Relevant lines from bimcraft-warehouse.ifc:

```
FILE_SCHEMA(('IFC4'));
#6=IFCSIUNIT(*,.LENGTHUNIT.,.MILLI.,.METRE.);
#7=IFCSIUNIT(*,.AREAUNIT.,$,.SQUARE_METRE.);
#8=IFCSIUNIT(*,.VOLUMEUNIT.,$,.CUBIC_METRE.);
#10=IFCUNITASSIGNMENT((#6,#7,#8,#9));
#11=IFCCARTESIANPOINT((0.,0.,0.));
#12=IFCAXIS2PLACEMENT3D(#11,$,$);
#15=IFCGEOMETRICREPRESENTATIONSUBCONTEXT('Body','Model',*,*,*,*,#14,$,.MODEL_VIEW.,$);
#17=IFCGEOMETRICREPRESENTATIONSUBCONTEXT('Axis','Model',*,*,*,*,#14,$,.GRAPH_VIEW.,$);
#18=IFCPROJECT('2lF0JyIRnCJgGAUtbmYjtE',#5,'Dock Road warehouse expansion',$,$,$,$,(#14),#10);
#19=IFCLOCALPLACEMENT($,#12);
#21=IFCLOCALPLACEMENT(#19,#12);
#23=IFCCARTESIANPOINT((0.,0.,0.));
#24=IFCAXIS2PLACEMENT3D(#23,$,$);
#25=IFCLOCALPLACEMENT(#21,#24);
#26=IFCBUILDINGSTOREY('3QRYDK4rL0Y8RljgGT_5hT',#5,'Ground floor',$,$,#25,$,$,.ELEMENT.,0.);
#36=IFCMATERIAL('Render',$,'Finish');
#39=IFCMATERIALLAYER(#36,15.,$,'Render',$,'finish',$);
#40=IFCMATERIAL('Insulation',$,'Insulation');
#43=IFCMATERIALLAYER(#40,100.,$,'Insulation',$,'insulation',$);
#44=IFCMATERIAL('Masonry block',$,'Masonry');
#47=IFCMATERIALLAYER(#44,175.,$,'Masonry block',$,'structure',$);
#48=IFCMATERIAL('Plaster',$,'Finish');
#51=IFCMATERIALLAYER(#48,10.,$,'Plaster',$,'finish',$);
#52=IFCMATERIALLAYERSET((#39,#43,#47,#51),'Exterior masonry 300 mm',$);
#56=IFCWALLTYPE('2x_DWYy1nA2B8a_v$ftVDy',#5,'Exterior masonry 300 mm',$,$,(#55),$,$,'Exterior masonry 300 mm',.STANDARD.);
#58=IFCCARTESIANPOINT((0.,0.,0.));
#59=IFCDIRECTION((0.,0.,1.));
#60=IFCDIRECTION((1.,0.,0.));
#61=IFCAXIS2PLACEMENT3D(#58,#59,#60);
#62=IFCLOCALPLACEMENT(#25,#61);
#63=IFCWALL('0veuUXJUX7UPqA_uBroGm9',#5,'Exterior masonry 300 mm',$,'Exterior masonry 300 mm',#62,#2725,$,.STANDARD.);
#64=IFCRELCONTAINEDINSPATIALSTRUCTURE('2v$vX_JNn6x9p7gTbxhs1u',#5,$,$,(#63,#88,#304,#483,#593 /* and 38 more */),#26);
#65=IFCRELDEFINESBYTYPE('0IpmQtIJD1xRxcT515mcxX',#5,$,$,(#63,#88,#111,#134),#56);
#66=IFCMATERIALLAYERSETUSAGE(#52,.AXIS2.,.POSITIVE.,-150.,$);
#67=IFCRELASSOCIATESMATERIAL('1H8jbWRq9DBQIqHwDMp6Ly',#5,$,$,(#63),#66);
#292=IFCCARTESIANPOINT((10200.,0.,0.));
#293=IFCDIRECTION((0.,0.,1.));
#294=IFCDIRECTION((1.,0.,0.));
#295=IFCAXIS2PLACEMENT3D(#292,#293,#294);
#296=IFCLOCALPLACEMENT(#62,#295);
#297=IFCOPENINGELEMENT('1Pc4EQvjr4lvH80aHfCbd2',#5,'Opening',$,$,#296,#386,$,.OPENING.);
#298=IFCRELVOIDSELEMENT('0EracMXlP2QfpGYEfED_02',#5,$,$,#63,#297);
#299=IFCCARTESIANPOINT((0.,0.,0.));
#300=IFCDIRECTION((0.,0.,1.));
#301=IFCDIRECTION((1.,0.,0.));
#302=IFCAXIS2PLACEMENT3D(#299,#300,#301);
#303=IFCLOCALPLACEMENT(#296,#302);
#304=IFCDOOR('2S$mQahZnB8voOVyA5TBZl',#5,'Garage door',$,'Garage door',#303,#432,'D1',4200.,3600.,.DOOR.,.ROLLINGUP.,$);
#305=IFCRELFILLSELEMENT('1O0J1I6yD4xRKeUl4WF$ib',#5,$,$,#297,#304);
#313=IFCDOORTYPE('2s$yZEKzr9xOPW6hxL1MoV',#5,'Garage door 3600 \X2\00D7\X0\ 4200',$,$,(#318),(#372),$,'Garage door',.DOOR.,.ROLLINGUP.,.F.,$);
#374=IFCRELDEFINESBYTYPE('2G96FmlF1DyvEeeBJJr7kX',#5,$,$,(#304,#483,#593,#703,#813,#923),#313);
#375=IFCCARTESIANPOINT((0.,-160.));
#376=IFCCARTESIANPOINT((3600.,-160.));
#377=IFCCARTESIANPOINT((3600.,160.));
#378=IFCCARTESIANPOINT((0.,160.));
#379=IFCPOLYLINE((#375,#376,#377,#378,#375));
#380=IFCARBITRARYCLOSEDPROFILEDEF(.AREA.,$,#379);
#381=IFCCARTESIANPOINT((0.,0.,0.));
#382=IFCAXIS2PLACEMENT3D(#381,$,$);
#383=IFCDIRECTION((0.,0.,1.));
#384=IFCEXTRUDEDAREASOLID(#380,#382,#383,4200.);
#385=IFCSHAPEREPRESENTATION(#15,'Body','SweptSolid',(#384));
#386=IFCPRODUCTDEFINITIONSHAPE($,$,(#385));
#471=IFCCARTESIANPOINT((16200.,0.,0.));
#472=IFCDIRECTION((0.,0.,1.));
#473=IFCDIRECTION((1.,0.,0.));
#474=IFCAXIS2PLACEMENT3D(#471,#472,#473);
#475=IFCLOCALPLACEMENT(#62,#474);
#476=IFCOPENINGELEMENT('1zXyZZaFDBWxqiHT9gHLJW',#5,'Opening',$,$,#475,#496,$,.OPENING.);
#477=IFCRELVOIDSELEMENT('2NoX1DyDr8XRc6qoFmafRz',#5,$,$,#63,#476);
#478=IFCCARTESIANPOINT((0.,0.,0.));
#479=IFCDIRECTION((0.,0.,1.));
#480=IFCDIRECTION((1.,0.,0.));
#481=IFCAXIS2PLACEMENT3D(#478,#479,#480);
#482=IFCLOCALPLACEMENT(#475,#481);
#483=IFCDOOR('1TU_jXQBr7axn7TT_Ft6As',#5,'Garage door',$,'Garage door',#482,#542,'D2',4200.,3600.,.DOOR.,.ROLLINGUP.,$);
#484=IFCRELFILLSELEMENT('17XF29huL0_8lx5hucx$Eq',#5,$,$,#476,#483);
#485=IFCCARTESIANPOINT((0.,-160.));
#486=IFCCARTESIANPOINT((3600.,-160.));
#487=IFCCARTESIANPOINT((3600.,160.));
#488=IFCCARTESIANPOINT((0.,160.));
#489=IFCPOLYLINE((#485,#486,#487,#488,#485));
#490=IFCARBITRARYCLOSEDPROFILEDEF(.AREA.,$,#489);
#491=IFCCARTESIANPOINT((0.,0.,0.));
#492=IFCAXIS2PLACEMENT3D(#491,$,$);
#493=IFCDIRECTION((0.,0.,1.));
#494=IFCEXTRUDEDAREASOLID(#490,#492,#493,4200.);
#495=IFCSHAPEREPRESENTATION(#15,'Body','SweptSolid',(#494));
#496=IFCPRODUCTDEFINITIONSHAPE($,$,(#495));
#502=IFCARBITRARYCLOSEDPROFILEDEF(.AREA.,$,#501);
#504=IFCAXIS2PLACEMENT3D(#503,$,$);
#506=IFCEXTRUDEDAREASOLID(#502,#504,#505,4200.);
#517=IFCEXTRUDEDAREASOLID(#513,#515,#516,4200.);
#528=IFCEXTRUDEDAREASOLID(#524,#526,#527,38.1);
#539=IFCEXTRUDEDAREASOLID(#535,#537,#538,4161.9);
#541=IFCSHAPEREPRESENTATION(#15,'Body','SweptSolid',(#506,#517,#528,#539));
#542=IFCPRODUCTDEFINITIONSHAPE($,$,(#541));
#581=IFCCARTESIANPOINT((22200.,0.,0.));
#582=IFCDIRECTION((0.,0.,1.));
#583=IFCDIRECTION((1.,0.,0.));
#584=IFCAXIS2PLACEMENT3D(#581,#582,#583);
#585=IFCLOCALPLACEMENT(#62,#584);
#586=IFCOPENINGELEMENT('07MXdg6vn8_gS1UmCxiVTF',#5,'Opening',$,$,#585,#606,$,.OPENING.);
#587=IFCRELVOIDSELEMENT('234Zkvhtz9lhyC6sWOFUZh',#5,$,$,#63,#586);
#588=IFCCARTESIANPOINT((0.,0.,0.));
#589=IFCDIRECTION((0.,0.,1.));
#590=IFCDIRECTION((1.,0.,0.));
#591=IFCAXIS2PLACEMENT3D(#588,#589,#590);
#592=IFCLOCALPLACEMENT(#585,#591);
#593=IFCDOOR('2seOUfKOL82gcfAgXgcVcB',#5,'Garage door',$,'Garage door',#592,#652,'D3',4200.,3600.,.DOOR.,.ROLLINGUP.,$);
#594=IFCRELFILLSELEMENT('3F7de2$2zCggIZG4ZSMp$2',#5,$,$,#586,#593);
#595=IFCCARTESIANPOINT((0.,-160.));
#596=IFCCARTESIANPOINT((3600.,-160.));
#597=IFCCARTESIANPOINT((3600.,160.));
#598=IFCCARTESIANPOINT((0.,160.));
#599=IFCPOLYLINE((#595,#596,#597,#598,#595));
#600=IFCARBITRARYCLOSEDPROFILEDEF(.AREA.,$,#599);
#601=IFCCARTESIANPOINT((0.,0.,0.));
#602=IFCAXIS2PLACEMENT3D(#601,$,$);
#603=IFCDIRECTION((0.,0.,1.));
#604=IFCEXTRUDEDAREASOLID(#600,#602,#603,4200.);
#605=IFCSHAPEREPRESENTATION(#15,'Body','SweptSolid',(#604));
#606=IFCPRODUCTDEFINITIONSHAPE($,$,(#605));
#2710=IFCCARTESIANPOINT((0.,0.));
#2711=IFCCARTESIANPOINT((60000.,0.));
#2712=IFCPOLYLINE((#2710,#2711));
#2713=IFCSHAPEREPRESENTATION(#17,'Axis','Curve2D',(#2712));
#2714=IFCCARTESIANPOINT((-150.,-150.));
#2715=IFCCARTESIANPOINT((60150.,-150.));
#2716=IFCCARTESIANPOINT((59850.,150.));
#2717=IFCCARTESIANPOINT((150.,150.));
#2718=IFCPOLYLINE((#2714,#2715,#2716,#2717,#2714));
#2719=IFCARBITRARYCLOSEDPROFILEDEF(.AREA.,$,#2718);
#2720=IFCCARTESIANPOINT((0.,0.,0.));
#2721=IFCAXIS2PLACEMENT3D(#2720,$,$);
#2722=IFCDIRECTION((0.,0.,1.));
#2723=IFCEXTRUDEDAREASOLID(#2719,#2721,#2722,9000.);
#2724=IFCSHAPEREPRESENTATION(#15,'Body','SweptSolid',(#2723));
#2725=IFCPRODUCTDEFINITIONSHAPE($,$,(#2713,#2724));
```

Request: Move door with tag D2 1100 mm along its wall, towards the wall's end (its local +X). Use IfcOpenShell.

```python
import ifcopenshell
import ifcopenshell.api.geometry
import ifcopenshell.util.placement

model = ifcopenshell.open("bimcraft-warehouse.ifc")

door = model.by_guid("1TU_jXQBr7axn7TT_Ft6As")
opening = door.FillsVoids[0].RelatingOpeningElement
wall = opening.VoidsElements[0].RelatingBuildingElement

wall_matrix = ifcopenshell.util.placement.get_local_placement(wall.ObjectPlacement)
shift = wall_matrix[:3, 0] * 1100.0
before = ifcopenshell.util.placement.get_local_placement(door.ObjectPlacement)[:3, 3].copy()

# The door is placed relative to its opening, so it follows when the opening moves.
matrix = ifcopenshell.util.placement.get_local_placement(opening.ObjectPlacement)
matrix[:3, 3] += shift
ifcopenshell.api.geometry.edit_object_placement(
    model, product=opening, matrix=matrix, is_si=False, should_transform_children=True
)

after = ifcopenshell.util.placement.get_local_placement(door.ObjectPlacement)[:3, 3]
print("door moved by", (after - before).round(3) + 0.0)

model.write("bimcraft-warehouse_v2.ifc")
```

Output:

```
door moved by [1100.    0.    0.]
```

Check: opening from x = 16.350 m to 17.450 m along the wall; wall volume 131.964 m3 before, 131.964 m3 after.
